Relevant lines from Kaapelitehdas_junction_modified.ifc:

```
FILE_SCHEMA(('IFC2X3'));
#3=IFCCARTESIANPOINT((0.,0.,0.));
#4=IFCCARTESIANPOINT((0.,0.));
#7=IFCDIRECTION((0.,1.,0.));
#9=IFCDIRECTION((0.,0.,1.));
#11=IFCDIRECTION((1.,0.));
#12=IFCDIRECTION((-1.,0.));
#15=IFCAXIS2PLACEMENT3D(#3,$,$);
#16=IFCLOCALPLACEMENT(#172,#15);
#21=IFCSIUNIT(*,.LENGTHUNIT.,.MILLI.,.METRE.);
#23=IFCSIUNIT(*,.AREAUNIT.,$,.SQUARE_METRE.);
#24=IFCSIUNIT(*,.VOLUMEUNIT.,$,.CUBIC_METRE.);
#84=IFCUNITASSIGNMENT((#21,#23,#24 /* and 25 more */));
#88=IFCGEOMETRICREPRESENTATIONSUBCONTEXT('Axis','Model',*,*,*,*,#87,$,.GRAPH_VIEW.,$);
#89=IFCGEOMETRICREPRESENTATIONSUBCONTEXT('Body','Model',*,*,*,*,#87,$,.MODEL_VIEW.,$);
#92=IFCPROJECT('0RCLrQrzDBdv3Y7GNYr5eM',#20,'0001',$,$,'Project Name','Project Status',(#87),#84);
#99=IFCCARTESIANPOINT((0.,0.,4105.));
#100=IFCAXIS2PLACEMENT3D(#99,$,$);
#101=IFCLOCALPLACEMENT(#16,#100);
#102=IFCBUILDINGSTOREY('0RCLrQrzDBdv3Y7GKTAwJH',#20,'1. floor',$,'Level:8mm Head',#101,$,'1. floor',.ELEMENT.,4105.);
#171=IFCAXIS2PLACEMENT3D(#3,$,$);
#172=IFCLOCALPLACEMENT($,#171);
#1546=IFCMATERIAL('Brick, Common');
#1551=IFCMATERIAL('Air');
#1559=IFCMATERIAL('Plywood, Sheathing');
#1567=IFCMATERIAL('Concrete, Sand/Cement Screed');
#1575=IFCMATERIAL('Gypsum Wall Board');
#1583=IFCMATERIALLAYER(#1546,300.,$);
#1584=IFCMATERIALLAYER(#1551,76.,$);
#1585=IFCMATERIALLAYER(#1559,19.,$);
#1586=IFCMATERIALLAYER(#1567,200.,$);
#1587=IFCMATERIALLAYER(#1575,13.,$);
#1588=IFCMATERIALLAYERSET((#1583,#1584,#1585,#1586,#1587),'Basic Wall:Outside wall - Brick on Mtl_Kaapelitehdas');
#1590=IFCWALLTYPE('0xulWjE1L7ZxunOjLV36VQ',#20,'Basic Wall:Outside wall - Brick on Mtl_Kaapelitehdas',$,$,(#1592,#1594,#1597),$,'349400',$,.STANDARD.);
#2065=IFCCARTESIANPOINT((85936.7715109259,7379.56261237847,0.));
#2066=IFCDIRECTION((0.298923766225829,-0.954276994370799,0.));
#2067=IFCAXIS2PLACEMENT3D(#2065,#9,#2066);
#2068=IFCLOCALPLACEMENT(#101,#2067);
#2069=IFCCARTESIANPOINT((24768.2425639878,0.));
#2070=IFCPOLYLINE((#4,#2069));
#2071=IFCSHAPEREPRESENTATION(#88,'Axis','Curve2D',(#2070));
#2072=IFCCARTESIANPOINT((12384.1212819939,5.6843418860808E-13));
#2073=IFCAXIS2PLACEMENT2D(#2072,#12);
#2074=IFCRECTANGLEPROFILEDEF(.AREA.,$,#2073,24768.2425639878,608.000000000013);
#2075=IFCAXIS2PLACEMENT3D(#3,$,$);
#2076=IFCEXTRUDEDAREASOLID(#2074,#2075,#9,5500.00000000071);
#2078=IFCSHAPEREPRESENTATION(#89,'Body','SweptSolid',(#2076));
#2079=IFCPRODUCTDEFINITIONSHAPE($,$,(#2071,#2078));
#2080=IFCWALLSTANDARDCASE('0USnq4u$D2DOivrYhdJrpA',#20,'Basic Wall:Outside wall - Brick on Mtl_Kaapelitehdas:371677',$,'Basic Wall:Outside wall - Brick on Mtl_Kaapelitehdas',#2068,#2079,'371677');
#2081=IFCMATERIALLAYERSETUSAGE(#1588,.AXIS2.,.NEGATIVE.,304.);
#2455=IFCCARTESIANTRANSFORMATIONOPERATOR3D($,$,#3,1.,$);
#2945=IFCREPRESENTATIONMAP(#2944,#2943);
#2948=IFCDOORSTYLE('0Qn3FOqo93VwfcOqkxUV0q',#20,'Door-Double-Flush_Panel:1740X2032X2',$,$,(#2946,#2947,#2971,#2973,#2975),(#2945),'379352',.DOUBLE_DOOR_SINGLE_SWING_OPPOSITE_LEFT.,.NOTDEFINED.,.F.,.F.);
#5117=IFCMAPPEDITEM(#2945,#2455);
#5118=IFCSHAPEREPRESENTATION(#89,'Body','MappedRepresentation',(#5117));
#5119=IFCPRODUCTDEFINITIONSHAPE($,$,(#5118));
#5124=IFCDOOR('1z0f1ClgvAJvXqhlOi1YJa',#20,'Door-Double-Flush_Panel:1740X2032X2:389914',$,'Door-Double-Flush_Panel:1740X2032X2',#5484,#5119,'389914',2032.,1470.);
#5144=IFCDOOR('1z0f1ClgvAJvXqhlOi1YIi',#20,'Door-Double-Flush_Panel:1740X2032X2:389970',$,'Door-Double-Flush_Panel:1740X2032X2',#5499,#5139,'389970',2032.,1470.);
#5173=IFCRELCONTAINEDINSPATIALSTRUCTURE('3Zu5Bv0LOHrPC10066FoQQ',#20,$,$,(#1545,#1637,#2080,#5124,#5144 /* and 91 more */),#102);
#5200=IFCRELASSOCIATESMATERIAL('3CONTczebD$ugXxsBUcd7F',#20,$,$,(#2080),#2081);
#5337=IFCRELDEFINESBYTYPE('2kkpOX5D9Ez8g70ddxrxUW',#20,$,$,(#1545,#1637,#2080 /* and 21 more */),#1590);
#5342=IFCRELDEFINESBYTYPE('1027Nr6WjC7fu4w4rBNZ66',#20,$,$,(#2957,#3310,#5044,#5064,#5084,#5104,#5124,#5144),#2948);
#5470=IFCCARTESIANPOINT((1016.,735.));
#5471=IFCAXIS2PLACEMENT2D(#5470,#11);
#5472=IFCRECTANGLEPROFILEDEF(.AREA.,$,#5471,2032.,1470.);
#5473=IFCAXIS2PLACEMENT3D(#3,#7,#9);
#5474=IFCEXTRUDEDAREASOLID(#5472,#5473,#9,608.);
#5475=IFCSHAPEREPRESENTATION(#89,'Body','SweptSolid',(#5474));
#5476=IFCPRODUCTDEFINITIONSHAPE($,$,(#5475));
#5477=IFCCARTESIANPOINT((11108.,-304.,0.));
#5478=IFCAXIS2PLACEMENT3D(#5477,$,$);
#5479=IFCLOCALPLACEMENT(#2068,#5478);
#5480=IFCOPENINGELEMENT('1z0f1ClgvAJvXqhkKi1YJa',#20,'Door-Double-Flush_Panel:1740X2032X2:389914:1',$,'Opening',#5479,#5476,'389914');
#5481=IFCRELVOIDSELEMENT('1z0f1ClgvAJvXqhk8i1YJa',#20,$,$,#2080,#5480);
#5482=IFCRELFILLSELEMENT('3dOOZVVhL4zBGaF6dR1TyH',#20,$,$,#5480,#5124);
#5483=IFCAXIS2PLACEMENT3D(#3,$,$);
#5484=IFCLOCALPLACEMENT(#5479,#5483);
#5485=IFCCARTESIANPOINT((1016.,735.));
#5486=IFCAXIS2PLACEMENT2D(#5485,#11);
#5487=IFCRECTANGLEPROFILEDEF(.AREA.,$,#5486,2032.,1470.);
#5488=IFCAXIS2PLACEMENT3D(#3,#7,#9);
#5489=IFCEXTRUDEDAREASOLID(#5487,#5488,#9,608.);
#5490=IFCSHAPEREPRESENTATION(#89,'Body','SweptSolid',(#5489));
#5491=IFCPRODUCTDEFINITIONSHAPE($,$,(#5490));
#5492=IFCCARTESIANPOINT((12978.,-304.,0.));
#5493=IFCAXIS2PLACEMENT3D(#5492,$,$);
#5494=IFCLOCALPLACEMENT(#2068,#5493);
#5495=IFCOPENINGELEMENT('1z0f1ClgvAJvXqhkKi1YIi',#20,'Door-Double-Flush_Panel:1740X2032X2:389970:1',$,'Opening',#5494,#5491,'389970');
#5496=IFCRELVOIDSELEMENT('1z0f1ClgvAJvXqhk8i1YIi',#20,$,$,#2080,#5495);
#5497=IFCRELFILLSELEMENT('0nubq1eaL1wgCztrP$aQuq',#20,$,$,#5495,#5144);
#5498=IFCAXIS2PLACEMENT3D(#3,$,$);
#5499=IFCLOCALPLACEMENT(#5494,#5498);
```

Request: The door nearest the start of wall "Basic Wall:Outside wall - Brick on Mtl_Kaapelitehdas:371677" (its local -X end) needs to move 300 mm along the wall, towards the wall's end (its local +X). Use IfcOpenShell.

```python
import ifcopenshell
import ifcopenshell.api.geometry
import ifcopenshell.util.placement
import ifcopenshell.util.unit

model = ifcopenshell.open("Kaapelitehdas_junction_modified.ifc")
unit_scale = ifcopenshell.util.unit.calculate_unit_scale(model)

door = model.by_guid("1z0f1ClgvAJvXqhlOi1YJa")
opening = door.FillsVoids[0].RelatingOpeningElement
wall = opening.VoidsElements[0].RelatingBuildingElement

wall_matrix = ifcopenshell.util.placement.get_local_placement(wall.ObjectPlacement)
shift = wall_matrix[:3, 0] * 0.3 / unit_scale
before = ifcopenshell.util.placement.get_local_placement(door.ObjectPlacement)[:3, 3].copy()

# The door is placed relative to its opening, so it follows when the opening moves.
matrix = ifcopenshell.util.placement.get_local_placement(opening.ObjectPlacement)
matrix[:3, 3] += shift
ifcopenshell.api.geometry.edit_object_placement(
    model, product=opening, matrix=matrix, is_si=False, should_transform_children=True
)

after = ifcopenshell.util.placement.get_local_placement(door.ObjectPlacement)[:3, 3]
print("door moved by", (after - before).round(3) + 0.0)

model.write("Kaapelitehdas_junction_modified_updated.ifc")
```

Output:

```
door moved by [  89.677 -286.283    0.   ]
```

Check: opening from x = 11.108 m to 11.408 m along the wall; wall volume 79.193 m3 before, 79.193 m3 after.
